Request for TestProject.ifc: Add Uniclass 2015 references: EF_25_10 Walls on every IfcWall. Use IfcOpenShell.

First a look at what the model holds.

```python
import ifcopenshell

model = ifcopenshell.open("TestProject.ifc")
print(model.schema)
print("classifications:", [c.Name for c in model.by_type("IfcClassification")])
for ifc_class in ("IfcDoor", "IfcRoof", "IfcStair", "IfcWall", "IfcWindow"):
    print(ifc_class, len(model.by_type(ifc_class)))
```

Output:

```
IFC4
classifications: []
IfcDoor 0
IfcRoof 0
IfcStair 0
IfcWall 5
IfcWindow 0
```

```python
import ifcopenshell
import ifcopenshell.api.classification

model = ifcopenshell.open("TestProject.ifc")

system = ifcopenshell.api.classification.add_classification(model, classification="Uniclass 2015")

codes = {
    "IfcWall": ("EF_25_10", "Walls"),
}
for ifc_class, (code, name) in codes.items():
    products = model.by_type(ifc_class)
    ifcopenshell.api.classification.add_reference(
        model, products=products, classification=system, identification=code, name=name
    )
    print(code, len(products))

model.write("TestProject_rev.ifc")
```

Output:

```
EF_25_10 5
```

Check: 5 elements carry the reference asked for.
